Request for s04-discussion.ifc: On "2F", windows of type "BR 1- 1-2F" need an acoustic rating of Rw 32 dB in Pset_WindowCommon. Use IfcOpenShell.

First a look at what the model holds.

```python
import ifcopenshell
import ifcopenshell.util.element

model = ifcopenshell.open("s04-discussion.ifc")
print(model.schema)
storey = next(s for s in model.by_type("IfcBuildingStorey") if s.Name == "2F")
windows = [e for e in ifcopenshell.util.element.get_decomposition(storey) if e.is_a("IfcWindow")]
seen = {}
for e in windows:
    element_type = ifcopenshell.util.element.get_type(e)
    key = (element_type.Name if element_type != e and element_type else None, ifcopenshell.util.element.get_pset(e, "Pset_WindowCommon", "AcousticRating"))
    seen[key] = seen.get(key, 0) + 1
for (name, value), count in sorted(seen.items(), key=str):
    print(count, "x", name, "|", value)
```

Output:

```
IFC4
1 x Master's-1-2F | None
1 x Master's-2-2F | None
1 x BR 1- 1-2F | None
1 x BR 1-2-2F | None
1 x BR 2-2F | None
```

```python
import ifcopenshell
import ifcopenshell.api.pset
import ifcopenshell.util.element

model = ifcopenshell.open("s04-discussion.ifc")

storey = next(s for s in model.by_type("IfcBuildingStorey") if s.Name == "2F")
windows = [e for e in ifcopenshell.util.element.get_decomposition(storey) if e.is_a("IfcWindow")]

count = 0
for e in windows:
    element_type = ifcopenshell.util.element.get_type(e)
    if element_type in (None, e) or element_type.Name != "BR 1- 1-2F":
        continue
    # add_pset returns the element's existing set when there is one.
    pset = ifcopenshell.api.pset.add_pset(model, product=e, name="Pset_WindowCommon")
    ifcopenshell.api.pset.edit_pset(model, pset=pset, properties={"AcousticRating": "Rw 32 dB"})
    count += 1

print(count, "windows updated")

model.write("s04-discussion_rev.ifc")
```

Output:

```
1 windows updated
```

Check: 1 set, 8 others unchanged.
